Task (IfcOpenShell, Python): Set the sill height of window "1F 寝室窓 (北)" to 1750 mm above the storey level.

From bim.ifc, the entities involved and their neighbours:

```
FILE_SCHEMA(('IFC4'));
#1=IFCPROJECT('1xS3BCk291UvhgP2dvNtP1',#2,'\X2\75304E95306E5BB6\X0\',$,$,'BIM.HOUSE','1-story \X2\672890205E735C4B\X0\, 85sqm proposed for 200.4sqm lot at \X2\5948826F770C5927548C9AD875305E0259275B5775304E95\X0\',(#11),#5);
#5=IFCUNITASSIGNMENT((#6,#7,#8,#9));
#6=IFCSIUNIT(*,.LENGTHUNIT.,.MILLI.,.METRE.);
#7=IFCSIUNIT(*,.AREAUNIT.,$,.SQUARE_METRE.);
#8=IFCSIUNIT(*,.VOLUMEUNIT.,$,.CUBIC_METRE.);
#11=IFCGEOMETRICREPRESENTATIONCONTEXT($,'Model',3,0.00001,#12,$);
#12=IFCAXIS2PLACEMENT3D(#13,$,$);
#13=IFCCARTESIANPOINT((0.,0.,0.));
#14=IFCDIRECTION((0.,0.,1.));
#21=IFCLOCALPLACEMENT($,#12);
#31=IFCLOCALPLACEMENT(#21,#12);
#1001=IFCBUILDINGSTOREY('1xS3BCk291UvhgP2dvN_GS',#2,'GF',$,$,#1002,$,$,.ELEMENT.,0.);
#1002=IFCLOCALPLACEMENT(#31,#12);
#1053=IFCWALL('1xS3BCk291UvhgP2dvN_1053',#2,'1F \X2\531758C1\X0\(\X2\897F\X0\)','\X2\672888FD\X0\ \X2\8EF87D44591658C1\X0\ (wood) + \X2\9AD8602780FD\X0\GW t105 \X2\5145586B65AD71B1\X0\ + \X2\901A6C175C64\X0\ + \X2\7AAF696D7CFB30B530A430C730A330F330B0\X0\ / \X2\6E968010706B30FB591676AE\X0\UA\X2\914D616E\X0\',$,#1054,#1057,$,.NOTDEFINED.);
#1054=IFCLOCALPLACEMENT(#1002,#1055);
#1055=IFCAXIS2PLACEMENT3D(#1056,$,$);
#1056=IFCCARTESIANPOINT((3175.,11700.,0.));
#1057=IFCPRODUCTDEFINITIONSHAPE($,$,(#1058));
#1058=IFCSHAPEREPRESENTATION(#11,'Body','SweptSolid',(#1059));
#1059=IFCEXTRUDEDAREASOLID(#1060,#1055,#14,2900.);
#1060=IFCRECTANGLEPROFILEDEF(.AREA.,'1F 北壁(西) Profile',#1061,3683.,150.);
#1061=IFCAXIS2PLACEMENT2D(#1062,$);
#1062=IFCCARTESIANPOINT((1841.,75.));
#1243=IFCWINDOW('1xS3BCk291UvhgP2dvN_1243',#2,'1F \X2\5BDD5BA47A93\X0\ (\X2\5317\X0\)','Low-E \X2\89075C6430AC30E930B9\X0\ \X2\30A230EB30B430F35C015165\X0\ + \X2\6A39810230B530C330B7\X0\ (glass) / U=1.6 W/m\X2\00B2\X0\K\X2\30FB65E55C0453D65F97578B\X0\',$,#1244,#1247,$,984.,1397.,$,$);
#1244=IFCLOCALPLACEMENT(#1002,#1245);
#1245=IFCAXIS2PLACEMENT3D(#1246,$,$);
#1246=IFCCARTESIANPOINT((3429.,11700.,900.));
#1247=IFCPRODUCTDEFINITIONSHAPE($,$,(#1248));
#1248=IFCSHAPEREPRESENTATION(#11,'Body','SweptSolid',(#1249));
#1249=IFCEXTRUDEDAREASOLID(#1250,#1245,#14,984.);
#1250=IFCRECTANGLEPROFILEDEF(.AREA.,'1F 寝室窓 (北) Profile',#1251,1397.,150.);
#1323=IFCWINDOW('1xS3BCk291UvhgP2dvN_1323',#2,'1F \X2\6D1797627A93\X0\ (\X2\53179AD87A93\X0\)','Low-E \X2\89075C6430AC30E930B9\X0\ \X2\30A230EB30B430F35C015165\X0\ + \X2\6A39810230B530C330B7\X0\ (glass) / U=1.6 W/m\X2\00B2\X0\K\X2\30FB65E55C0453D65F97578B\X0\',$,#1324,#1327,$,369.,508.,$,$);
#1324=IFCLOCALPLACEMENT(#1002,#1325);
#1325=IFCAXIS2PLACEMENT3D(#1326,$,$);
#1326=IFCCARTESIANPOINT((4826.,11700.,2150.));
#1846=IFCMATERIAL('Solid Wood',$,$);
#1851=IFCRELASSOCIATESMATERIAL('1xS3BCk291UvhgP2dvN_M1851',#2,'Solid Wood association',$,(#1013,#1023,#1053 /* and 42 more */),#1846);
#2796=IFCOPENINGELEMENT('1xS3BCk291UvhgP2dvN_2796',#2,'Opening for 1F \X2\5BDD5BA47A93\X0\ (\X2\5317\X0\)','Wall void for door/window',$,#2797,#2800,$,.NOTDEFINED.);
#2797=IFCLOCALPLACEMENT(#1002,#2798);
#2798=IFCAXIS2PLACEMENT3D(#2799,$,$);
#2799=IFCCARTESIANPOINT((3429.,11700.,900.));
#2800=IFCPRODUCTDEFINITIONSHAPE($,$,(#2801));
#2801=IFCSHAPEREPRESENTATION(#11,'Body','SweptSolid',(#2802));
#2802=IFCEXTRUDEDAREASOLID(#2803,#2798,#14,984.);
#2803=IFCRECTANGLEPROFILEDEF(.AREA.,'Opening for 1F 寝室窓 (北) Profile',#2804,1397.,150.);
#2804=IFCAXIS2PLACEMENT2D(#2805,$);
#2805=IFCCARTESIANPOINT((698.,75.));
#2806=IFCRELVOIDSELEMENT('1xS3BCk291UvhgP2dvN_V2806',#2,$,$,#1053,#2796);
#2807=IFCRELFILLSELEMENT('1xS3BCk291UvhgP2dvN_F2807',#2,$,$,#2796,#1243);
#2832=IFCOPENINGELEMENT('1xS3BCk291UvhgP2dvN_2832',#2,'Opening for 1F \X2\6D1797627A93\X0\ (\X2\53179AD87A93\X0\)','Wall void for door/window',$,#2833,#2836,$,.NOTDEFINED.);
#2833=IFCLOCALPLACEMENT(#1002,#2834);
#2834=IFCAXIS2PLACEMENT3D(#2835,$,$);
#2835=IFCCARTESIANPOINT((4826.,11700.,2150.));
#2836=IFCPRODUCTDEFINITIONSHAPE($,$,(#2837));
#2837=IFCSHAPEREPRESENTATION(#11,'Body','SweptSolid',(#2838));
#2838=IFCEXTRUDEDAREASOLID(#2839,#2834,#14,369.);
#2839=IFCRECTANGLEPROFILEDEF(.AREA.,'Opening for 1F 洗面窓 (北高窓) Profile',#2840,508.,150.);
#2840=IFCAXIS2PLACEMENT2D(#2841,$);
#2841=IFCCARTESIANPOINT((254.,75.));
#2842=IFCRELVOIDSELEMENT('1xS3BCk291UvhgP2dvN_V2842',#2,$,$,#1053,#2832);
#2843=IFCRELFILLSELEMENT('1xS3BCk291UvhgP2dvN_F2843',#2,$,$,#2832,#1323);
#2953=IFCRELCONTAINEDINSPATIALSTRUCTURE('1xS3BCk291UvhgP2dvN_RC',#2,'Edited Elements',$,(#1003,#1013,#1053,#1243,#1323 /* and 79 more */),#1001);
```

```python
import numpy as np
import ifcopenshell
import ifcopenshell.api.geometry
import ifcopenshell.geom
import ifcopenshell.util.element
import ifcopenshell.util.placement
import ifcopenshell.util.shape
import ifcopenshell.util.unit

model = ifcopenshell.open("bim.ifc")
unit_scale = ifcopenshell.util.unit.calculate_unit_scale(model)

window = model.by_guid("1xS3BCk291UvhgP2dvN_1243")
opening = window.FillsVoids[0].RelatingOpeningElement
storey = ifcopenshell.util.element.get_container(window, ifc_class="IfcBuildingStorey")
level = ifcopenshell.util.placement.get_local_placement(storey.ObjectPlacement)[2, 3]

# The opening's origin need not be at the sill, so measure its lowest point.
shape = ifcopenshell.geom.create_shape(ifcopenshell.geom.settings(), opening)
bottom = ifcopenshell.util.shape.get_shape_bottom_elevation(shape, shape.geometry) / unit_scale
dz = level + 1750.0 - bottom

shift = np.array([0.0, 0.0, dz])
# The window is not placed relative to its opening, so move both.
for product in (opening, window):
    matrix = ifcopenshell.util.placement.get_local_placement(product.ObjectPlacement)
    matrix[:3, 3] += shift
    ifcopenshell.api.geometry.edit_object_placement(model, product=product, matrix=matrix, is_si=False)

print(f"moved by {dz * unit_scale:+.3f} m")

model.write("bim_edited.ifc")
```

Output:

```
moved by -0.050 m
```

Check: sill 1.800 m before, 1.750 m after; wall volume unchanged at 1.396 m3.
